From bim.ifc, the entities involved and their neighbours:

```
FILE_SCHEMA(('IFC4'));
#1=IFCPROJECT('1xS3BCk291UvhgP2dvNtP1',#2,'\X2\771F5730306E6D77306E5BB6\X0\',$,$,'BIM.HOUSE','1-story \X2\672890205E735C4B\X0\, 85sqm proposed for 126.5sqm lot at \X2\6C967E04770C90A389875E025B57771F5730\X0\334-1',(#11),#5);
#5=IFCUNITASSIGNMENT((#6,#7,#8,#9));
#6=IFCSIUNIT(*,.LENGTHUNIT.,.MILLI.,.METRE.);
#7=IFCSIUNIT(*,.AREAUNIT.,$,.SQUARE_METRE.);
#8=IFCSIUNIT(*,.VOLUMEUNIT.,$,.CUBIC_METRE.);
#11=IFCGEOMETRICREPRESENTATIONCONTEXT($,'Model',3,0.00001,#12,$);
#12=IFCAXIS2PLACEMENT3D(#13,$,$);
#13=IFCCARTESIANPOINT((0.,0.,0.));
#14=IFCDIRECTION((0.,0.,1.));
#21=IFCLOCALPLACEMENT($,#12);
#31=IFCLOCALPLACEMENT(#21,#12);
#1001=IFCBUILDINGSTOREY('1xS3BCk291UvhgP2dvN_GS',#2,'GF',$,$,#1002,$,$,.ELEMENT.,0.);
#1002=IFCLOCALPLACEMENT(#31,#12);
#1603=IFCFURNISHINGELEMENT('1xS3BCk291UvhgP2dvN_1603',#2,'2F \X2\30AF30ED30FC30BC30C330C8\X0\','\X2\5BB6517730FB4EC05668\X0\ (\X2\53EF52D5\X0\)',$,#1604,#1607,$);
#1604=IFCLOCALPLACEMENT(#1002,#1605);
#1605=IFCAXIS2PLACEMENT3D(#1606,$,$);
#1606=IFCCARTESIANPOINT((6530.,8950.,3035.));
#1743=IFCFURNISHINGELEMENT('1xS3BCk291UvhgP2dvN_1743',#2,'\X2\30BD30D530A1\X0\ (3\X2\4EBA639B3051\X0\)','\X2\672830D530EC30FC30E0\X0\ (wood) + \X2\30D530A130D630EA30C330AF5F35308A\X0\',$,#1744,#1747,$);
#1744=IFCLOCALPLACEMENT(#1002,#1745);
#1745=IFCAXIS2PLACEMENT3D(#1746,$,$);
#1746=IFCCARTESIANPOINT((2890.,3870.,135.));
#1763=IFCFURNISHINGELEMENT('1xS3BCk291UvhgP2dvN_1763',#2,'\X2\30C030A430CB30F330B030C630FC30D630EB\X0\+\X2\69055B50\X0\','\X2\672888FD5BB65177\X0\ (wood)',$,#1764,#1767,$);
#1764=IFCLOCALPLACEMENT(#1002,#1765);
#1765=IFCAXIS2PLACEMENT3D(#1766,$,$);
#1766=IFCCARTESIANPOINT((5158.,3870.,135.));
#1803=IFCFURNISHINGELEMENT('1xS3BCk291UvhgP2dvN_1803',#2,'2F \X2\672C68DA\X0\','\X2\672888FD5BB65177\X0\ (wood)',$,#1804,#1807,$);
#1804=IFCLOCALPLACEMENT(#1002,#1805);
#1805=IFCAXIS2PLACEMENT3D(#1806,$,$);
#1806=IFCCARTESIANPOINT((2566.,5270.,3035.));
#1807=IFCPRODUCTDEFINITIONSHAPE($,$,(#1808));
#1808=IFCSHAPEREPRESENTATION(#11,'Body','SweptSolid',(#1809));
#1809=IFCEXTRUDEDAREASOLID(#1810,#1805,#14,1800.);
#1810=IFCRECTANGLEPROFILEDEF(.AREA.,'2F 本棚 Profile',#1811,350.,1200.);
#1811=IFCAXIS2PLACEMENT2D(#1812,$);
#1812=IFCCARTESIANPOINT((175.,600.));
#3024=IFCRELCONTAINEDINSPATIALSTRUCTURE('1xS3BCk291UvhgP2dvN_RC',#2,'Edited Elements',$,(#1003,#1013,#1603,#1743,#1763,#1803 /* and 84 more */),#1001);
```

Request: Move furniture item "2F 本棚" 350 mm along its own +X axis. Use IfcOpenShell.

```python
import ifcopenshell
import ifcopenshell.api.geometry
import ifcopenshell.util.placement

model = ifcopenshell.open("bim.ifc")

item = model.by_guid("1xS3BCk291UvhgP2dvN_1803")
matrix = ifcopenshell.util.placement.get_local_placement(item.ObjectPlacement)
matrix[:3, 3] += matrix[:3, 0] * 350.0
ifcopenshell.api.geometry.edit_object_placement(model, product=item, matrix=matrix, is_si=False)

print(ifcopenshell.util.placement.get_local_placement(item.ObjectPlacement).round(3) + 0.0)

model.write("bim_updated.ifc")
```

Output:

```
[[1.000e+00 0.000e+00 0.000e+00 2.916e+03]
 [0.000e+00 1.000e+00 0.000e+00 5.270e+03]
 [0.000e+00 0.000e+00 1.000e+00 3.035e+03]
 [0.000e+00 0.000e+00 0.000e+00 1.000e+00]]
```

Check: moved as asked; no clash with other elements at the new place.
